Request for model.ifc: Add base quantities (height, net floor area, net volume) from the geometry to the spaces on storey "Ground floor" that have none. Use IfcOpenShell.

First a look at what the model holds.

```python
import ifcopenshell
import ifcopenshell.util.element
import ifcopenshell.util.unit

model = ifcopenshell.open("model.ifc")
print(model.schema)
for unit_type in ("LENGTHUNIT", "AREAUNIT", "VOLUMEUNIT"):
    print(unit_type, ifcopenshell.util.unit.calculate_unit_scale(model, unit_type))
storey = next(s for s in model.by_type("IfcBuildingStorey") if s.Name == "Ground floor")
spaces = [e for e in ifcopenshell.util.element.get_decomposition(storey) if e.is_a("IfcSpace")]
for e in sorted(spaces, key=lambda e: e.id()):
    print(e.id(), e.is_a(), e.Name, list(ifcopenshell.util.element.get_psets(e, qtos_only=True)), sep=" | ")
```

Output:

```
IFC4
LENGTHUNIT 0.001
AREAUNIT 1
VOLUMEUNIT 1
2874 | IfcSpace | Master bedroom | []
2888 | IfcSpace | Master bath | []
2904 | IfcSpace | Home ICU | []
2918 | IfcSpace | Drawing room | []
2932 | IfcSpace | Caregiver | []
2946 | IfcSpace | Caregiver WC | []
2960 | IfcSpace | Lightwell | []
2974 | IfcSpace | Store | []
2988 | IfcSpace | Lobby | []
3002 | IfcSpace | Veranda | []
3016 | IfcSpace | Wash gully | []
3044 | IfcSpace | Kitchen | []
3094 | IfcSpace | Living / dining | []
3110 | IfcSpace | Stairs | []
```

```python
import ifcopenshell
import ifcopenshell.api.pset
import ifcopenshell.geom
import ifcopenshell.util.element
import ifcopenshell.util.shape
import ifcopenshell.util.unit

model = ifcopenshell.open("model.ifc")
unit_scale = ifcopenshell.util.unit.calculate_unit_scale(model)
area_scale = ifcopenshell.util.unit.calculate_unit_scale(model, "AREAUNIT")
volume_scale = ifcopenshell.util.unit.calculate_unit_scale(model, "VOLUMEUNIT")
settings = ifcopenshell.geom.settings()

storey = next(s for s in model.by_type("IfcBuildingStorey") if s.Name == "Ground floor")
spaces = [e for e in ifcopenshell.util.element.get_decomposition(storey) if e.is_a("IfcSpace")]

for e in sorted(spaces, key=lambda e: e.id()):
    if ifcopenshell.util.element.get_psets(e, qtos_only=True, should_inherit=False):
        continue
    # Geometry comes back in metres, in the element's own axes.
    shape = ifcopenshell.geom.create_shape(settings, e)
    values = {
        "Height": ifcopenshell.util.shape.get_z(shape.geometry) / unit_scale,
        "NetFloorArea": ifcopenshell.util.shape.get_footprint_area(shape.geometry) / area_scale,
        "NetVolume": ifcopenshell.util.shape.get_volume(shape.geometry) / volume_scale,
    }
    qto = ifcopenshell.api.pset.add_qto(model, product=e, name="Qto_SpaceBaseQuantities")
    ifcopenshell.api.pset.edit_qto(model, qto=qto, properties=values)
    print(e.id(), {k: round(v, 3) for k, v in values.items()})

model.write("model_updated.ifc")
```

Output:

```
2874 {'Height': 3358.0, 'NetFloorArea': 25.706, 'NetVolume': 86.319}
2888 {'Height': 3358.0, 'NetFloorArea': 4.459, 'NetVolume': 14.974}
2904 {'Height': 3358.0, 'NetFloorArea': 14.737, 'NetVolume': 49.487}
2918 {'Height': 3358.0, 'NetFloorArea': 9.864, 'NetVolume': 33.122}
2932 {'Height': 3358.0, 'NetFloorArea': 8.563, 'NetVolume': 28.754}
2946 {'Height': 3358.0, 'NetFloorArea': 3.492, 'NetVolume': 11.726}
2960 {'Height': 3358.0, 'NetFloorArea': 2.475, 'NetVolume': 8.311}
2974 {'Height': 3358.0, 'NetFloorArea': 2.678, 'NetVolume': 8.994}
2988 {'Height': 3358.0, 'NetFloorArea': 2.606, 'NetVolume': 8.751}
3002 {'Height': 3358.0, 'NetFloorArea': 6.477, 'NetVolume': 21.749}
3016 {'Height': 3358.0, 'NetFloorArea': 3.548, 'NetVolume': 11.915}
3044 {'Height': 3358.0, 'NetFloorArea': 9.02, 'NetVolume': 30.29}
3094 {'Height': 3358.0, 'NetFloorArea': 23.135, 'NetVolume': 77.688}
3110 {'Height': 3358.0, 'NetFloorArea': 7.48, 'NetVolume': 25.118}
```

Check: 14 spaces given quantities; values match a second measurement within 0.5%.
